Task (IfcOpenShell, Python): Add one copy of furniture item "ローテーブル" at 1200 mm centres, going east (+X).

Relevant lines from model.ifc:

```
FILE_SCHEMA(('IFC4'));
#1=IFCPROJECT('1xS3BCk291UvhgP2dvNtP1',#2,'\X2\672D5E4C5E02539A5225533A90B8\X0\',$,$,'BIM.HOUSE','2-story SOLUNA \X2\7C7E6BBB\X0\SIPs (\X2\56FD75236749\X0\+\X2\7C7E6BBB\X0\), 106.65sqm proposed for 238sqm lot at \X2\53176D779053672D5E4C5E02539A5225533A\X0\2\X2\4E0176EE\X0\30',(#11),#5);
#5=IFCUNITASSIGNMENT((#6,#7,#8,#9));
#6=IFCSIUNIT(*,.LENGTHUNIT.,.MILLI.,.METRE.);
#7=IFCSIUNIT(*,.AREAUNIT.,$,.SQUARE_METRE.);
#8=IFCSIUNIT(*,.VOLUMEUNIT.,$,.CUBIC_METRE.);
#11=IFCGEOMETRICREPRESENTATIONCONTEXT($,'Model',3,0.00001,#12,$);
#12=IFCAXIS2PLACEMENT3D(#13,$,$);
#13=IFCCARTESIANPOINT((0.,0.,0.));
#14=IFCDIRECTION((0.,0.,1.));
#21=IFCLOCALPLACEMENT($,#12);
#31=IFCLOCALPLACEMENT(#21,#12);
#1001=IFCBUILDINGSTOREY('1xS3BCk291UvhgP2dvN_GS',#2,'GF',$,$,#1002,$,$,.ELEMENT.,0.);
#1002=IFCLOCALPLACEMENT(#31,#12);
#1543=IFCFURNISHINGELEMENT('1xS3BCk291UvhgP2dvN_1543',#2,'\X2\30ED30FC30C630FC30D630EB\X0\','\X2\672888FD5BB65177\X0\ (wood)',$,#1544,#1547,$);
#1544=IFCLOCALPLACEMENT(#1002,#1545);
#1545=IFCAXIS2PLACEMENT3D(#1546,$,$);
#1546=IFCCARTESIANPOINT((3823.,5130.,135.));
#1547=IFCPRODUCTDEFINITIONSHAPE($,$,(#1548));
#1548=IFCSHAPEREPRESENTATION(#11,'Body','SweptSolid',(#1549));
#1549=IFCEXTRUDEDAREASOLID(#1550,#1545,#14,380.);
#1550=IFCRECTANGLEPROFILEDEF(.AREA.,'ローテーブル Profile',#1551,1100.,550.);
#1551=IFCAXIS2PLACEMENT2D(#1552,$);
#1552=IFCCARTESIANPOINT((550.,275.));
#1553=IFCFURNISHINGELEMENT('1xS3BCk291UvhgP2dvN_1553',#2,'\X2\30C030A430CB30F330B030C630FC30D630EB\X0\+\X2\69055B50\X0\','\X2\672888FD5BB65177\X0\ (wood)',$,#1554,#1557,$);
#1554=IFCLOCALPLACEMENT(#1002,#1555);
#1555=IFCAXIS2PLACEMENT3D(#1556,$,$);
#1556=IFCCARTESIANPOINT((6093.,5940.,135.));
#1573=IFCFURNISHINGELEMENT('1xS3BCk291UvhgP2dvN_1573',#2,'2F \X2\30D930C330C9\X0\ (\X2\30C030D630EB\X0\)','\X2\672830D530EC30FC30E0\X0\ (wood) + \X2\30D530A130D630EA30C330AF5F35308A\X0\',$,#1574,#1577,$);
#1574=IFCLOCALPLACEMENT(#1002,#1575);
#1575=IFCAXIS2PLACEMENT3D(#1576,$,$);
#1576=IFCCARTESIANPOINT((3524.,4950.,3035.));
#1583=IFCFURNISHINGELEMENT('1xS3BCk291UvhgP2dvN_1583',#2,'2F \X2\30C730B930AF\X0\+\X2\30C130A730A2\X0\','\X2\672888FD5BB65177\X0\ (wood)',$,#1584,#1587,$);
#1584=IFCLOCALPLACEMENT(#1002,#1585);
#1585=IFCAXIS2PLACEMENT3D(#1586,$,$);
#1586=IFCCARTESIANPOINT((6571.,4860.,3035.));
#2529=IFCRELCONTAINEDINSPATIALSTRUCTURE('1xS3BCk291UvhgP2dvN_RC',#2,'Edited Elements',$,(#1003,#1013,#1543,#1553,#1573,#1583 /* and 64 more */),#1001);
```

```python
import numpy as np
import ifcopenshell
import ifcopenshell.api.geometry
import ifcopenshell.api.root
import ifcopenshell.util.element
import ifcopenshell.util.placement

model = ifcopenshell.open("model.ifc")


def reuse_history(source, copy):
    """copy_class also copies each property set's owner history, people and application; keep the originals."""
    for rel in copy.IsDefinedBy:
        if rel.is_a("IfcRelDefinesByProperties") and (history := rel.RelatingPropertyDefinition.OwnerHistory):
            rel.RelatingPropertyDefinition.OwnerHistory = source.OwnerHistory
            ifcopenshell.util.element.remove_deep2(model, history)


source = model.by_guid("1xS3BCk291UvhgP2dvN_1543")
base = ifcopenshell.util.placement.get_local_placement(source.ObjectPlacement)
step = np.array([1.0, 0.0, 0.0]) * 1200.0

for i in range(1, 2):
    copy = ifcopenshell.api.root.copy_class(model, product=source)
    copy.Representation = ifcopenshell.util.element.copy_deep(
        model, source.Representation, exclude=["IfcGeometricRepresentationContext", "IfcRepresentationMap"]
    )
    reuse_history(source, copy)
    matrix = base.copy()
    matrix[:3, 3] += i * step
    print("added at", matrix[:3, 3].round(3) + 0.0)
    ifcopenshell.api.geometry.edit_object_placement(model, product=copy, matrix=matrix, is_si=False)

model.write("model_v2.ifc")
```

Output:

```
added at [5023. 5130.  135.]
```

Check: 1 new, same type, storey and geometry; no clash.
